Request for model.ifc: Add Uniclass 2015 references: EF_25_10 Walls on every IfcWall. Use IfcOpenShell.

First a look at what the model holds.

```python
import ifcopenshell

model = ifcopenshell.open("model.ifc")
print(model.schema)
print("classifications:", [c.Name for c in model.by_type("IfcClassification")])
for ifc_class in ("IfcDoor", "IfcRoof", "IfcStair", "IfcWall", "IfcWindow"):
    print(ifc_class, len(model.by_type(ifc_class)))
```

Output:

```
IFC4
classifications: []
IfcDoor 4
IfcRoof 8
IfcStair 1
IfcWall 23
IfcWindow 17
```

```python
import ifcopenshell
import ifcopenshell.api.classification

model = ifcopenshell.open("model.ifc")

system = ifcopenshell.api.classification.add_classification(model, classification="Uniclass 2015")

codes = {
    "IfcWall": ("EF_25_10", "Walls"),
}
for ifc_class, (code, name) in codes.items():
    products = model.by_type(ifc_class)
    ifcopenshell.api.classification.add_reference(
        model, products=products, classification=system, identification=code, name=name
    )
    print(code, len(products))

model.write("model_rev.ifc")
```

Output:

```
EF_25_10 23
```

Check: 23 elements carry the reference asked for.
